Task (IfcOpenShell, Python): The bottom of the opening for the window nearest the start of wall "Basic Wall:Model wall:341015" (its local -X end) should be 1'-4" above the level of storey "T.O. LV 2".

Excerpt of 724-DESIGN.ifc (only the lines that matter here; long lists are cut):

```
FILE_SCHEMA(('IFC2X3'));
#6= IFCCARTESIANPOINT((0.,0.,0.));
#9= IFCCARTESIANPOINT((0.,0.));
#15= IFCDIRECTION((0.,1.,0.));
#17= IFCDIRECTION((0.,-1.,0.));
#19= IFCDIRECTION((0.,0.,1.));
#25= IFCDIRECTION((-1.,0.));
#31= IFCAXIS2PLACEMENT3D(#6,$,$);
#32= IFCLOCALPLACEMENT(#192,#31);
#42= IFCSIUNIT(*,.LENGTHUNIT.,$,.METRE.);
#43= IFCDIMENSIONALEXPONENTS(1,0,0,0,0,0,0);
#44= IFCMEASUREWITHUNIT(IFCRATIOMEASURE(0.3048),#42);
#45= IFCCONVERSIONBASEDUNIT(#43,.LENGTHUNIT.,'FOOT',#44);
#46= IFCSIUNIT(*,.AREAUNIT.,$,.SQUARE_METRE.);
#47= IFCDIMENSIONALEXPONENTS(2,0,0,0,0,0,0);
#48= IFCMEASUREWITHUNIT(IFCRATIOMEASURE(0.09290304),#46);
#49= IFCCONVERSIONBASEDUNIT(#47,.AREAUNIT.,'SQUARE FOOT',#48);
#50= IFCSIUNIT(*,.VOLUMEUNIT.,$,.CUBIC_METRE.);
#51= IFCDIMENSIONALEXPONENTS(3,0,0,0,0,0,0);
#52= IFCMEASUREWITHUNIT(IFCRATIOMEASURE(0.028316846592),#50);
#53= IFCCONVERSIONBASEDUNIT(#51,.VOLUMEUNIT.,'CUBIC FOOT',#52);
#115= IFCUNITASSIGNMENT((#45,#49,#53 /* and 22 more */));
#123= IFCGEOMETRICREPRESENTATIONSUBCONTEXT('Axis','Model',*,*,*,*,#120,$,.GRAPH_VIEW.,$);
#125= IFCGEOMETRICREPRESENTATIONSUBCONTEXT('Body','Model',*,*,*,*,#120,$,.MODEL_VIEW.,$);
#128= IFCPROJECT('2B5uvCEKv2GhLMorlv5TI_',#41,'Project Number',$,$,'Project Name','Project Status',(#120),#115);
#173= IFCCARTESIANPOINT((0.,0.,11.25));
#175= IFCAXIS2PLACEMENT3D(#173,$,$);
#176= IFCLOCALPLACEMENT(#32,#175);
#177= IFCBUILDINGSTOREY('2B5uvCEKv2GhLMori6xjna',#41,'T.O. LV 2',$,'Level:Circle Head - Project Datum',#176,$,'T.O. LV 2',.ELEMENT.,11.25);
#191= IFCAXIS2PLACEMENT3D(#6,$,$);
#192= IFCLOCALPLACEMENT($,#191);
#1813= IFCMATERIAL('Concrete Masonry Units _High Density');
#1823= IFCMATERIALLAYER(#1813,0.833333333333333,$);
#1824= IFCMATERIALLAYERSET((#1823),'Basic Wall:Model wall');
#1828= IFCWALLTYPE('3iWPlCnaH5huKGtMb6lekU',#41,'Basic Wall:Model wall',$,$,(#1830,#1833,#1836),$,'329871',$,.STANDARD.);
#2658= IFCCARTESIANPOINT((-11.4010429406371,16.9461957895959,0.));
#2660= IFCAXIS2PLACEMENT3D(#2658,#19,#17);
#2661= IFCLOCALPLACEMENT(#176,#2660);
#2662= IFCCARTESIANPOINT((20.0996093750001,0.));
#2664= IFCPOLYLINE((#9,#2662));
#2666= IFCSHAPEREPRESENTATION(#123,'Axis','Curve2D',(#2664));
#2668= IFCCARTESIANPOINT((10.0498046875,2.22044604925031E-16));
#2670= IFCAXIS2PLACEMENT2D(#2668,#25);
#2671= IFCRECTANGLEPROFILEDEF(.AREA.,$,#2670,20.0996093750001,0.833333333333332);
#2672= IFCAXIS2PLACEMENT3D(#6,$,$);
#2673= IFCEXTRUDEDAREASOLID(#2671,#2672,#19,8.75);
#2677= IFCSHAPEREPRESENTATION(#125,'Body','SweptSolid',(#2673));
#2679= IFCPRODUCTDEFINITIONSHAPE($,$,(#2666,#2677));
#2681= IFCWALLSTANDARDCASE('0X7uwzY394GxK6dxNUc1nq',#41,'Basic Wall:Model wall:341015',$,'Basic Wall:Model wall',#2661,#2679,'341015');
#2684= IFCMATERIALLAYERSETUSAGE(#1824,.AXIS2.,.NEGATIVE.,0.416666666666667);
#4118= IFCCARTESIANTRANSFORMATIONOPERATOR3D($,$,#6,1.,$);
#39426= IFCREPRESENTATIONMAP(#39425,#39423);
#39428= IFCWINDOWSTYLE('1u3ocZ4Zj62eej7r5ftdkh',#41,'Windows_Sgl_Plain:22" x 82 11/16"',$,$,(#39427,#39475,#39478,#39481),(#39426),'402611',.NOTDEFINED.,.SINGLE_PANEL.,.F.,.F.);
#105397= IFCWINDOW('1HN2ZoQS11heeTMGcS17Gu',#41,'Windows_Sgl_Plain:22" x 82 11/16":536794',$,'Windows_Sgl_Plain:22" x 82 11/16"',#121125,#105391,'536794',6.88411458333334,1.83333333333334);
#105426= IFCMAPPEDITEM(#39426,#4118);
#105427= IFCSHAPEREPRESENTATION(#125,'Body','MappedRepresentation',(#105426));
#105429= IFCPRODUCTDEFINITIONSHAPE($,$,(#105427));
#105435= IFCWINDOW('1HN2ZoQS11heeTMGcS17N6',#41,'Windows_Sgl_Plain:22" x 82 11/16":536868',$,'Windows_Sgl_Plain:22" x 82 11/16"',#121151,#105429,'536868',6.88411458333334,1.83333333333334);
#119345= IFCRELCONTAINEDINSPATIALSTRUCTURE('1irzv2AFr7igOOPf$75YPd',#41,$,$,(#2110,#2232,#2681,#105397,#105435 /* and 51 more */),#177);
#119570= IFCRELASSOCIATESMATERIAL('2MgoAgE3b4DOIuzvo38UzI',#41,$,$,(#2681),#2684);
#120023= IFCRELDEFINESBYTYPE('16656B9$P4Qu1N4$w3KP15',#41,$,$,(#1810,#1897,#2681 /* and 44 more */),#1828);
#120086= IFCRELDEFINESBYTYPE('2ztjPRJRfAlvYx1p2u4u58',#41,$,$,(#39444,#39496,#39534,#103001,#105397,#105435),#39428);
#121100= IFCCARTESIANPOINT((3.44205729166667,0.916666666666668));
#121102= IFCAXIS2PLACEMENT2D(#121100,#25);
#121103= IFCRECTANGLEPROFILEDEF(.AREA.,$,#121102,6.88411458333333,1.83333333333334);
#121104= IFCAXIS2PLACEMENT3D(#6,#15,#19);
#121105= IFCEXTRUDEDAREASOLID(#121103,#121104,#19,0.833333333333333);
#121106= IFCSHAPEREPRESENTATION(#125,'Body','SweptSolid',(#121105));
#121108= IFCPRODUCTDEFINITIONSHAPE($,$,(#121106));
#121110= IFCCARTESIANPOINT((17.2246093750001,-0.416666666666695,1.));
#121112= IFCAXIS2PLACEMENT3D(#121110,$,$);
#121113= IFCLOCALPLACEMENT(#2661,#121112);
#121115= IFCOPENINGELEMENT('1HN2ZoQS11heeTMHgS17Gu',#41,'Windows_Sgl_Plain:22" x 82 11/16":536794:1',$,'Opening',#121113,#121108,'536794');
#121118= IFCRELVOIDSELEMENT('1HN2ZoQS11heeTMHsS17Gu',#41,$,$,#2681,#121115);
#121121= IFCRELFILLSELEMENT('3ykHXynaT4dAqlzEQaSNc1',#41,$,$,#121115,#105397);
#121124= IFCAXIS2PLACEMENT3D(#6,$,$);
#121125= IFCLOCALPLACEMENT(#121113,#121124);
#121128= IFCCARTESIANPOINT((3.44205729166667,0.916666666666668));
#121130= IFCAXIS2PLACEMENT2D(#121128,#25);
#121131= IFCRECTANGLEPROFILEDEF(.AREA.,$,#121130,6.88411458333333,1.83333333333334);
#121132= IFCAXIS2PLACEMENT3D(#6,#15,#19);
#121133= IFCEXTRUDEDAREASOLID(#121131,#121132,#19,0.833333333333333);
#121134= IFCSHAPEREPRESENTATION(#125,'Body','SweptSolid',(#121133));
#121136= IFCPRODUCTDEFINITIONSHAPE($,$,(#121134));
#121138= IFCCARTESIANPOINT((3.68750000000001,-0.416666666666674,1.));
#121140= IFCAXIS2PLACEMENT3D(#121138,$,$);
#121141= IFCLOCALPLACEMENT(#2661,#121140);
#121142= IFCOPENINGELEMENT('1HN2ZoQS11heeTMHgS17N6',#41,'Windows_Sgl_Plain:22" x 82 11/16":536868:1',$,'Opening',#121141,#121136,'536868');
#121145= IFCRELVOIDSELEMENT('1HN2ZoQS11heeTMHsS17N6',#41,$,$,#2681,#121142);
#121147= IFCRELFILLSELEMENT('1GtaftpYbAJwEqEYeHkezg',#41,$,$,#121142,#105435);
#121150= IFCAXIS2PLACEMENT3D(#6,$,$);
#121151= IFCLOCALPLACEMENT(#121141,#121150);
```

```python
import numpy as np
import ifcopenshell
import ifcopenshell.api.geometry
import ifcopenshell.geom
import ifcopenshell.util.element
import ifcopenshell.util.placement
import ifcopenshell.util.shape
import ifcopenshell.util.unit

model = ifcopenshell.open("724-DESIGN.ifc")
unit_scale = ifcopenshell.util.unit.calculate_unit_scale(model)

window = model.by_guid("1HN2ZoQS11heeTMGcS17N6")
opening = window.FillsVoids[0].RelatingOpeningElement
storey = ifcopenshell.util.element.get_container(window, ifc_class="IfcBuildingStorey")
level = ifcopenshell.util.placement.get_local_placement(storey.ObjectPlacement)[2, 3]

# The opening's origin need not be at the sill, so measure its lowest point.
shape = ifcopenshell.geom.create_shape(ifcopenshell.geom.settings(), opening)
bottom = ifcopenshell.util.shape.get_shape_bottom_elevation(shape, shape.geometry) / unit_scale
dz = level + 16 * 0.0254 / unit_scale - bottom

shift = np.array([0.0, 0.0, dz])
# The window is placed relative to its opening, so it follows when the opening moves.
matrix = ifcopenshell.util.placement.get_local_placement(opening.ObjectPlacement)
matrix[:3, 3] += shift
ifcopenshell.api.geometry.edit_object_placement(
    model, product=opening, matrix=matrix, is_si=False, should_transform_children=True
)

print(f"moved by {dz * unit_scale:+.3f} m")

model.write("724-DESIGN_rev.ifc")
```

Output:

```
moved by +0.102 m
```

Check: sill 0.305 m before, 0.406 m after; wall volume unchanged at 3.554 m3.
